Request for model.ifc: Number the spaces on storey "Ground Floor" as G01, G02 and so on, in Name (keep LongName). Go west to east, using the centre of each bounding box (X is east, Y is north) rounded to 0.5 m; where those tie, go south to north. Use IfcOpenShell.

First a look at what the model holds.

```python
import ifcopenshell
import ifcopenshell.util.element
import ifcopenshell.util.placement

model = ifcopenshell.open("model.ifc")
print(model.schema)
storey = next(s for s in model.by_type("IfcBuildingStorey") if s.Name == "Ground Floor")
spaces = [e for e in ifcopenshell.util.element.get_decomposition(storey) if e.is_a("IfcSpace")]
for e in sorted(spaces, key=lambda e: e.id()):
    origin = ifcopenshell.util.placement.get_local_placement(e.ObjectPlacement)[:3, 3]
    print(e.id(), e.Name, e.LongName, origin.round(2) + 0.0, sep=" | ")
```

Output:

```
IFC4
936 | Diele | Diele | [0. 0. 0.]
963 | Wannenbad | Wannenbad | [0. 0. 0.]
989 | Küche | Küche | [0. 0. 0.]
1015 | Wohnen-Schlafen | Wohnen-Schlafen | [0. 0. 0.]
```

```python
import ifcopenshell
import ifcopenshell.geom
import ifcopenshell.util.element
import ifcopenshell.util.shape

model = ifcopenshell.open("model.ifc")
settings = ifcopenshell.geom.settings()
settings.set("use-world-coords", True)


def centre(element):
    shape = ifcopenshell.geom.create_shape(settings, element)
    return ifcopenshell.util.shape.get_bbox_centroid(shape.geometry)


storey = next(s for s in model.by_type("IfcBuildingStorey") if s.Name == "Ground Floor")
spaces = [e for e in ifcopenshell.util.element.get_decomposition(storey) if e.is_a("IfcSpace")]

# Insertion points can sit at a corner or the storey origin, so sort by the geometry (in metres).
centres = {e: centre(e) for e in spaces}
spaces.sort(key=lambda e: (round(centres[e][0] / 0.5), centres[e][1]))

for i, e in enumerate(spaces, start=1):
    number = f"G{i:02d}"
    e.Name = number
    print(e.id(), number)

model.write("model_edited.ifc")
```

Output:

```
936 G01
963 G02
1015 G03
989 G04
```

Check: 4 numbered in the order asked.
